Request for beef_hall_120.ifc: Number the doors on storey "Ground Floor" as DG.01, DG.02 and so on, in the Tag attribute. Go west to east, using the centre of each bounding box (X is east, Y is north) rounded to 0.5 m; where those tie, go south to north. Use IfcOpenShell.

First a look at what the model holds.

```python
import ifcopenshell
import ifcopenshell.util.element
import ifcopenshell.util.placement

model = ifcopenshell.open("beef_hall_120.ifc")
print(model.schema)
storey = next(s for s in model.by_type("IfcBuildingStorey") if s.Name == "Ground Floor")
doors = [e for e in ifcopenshell.util.element.get_decomposition(storey) if e.is_a("IfcDoor")]
for e in sorted(doors, key=lambda e: e.id()):
    origin = ifcopenshell.util.placement.get_local_placement(e.ObjectPlacement)[:3, 3]
    print(e.id(), e.Tag, e.Name, origin.round(2) + 0.0, sep=" | ")
```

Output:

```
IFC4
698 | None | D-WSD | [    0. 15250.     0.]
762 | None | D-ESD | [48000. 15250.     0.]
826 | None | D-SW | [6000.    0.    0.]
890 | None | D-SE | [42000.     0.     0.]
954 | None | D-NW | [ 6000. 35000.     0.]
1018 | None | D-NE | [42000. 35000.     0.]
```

```python
import ifcopenshell
import ifcopenshell.geom
import ifcopenshell.util.element
import ifcopenshell.util.shape

model = ifcopenshell.open("beef_hall_120.ifc")
settings = ifcopenshell.geom.settings()
settings.set("use-world-coords", True)


def centre(element):
    shape = ifcopenshell.geom.create_shape(settings, element)
    return ifcopenshell.util.shape.get_bbox_centroid(shape.geometry)


storey = next(s for s in model.by_type("IfcBuildingStorey") if s.Name == "Ground Floor")
doors = [e for e in ifcopenshell.util.element.get_decomposition(storey) if e.is_a("IfcDoor")]

# Insertion points can sit at a corner or the storey origin, so sort by the geometry (in metres).
centres = {e: centre(e) for e in doors}
doors.sort(key=lambda e: (round(centres[e][0] / 0.5), centres[e][1]))

for i, e in enumerate(doors, start=1):
    number = f"DG.{i:02d}"
    e.Tag = number
    print(e.id(), number)

model.write("beef_hall_120_edited.ifc")
```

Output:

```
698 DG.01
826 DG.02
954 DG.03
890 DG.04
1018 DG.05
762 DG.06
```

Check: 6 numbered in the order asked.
